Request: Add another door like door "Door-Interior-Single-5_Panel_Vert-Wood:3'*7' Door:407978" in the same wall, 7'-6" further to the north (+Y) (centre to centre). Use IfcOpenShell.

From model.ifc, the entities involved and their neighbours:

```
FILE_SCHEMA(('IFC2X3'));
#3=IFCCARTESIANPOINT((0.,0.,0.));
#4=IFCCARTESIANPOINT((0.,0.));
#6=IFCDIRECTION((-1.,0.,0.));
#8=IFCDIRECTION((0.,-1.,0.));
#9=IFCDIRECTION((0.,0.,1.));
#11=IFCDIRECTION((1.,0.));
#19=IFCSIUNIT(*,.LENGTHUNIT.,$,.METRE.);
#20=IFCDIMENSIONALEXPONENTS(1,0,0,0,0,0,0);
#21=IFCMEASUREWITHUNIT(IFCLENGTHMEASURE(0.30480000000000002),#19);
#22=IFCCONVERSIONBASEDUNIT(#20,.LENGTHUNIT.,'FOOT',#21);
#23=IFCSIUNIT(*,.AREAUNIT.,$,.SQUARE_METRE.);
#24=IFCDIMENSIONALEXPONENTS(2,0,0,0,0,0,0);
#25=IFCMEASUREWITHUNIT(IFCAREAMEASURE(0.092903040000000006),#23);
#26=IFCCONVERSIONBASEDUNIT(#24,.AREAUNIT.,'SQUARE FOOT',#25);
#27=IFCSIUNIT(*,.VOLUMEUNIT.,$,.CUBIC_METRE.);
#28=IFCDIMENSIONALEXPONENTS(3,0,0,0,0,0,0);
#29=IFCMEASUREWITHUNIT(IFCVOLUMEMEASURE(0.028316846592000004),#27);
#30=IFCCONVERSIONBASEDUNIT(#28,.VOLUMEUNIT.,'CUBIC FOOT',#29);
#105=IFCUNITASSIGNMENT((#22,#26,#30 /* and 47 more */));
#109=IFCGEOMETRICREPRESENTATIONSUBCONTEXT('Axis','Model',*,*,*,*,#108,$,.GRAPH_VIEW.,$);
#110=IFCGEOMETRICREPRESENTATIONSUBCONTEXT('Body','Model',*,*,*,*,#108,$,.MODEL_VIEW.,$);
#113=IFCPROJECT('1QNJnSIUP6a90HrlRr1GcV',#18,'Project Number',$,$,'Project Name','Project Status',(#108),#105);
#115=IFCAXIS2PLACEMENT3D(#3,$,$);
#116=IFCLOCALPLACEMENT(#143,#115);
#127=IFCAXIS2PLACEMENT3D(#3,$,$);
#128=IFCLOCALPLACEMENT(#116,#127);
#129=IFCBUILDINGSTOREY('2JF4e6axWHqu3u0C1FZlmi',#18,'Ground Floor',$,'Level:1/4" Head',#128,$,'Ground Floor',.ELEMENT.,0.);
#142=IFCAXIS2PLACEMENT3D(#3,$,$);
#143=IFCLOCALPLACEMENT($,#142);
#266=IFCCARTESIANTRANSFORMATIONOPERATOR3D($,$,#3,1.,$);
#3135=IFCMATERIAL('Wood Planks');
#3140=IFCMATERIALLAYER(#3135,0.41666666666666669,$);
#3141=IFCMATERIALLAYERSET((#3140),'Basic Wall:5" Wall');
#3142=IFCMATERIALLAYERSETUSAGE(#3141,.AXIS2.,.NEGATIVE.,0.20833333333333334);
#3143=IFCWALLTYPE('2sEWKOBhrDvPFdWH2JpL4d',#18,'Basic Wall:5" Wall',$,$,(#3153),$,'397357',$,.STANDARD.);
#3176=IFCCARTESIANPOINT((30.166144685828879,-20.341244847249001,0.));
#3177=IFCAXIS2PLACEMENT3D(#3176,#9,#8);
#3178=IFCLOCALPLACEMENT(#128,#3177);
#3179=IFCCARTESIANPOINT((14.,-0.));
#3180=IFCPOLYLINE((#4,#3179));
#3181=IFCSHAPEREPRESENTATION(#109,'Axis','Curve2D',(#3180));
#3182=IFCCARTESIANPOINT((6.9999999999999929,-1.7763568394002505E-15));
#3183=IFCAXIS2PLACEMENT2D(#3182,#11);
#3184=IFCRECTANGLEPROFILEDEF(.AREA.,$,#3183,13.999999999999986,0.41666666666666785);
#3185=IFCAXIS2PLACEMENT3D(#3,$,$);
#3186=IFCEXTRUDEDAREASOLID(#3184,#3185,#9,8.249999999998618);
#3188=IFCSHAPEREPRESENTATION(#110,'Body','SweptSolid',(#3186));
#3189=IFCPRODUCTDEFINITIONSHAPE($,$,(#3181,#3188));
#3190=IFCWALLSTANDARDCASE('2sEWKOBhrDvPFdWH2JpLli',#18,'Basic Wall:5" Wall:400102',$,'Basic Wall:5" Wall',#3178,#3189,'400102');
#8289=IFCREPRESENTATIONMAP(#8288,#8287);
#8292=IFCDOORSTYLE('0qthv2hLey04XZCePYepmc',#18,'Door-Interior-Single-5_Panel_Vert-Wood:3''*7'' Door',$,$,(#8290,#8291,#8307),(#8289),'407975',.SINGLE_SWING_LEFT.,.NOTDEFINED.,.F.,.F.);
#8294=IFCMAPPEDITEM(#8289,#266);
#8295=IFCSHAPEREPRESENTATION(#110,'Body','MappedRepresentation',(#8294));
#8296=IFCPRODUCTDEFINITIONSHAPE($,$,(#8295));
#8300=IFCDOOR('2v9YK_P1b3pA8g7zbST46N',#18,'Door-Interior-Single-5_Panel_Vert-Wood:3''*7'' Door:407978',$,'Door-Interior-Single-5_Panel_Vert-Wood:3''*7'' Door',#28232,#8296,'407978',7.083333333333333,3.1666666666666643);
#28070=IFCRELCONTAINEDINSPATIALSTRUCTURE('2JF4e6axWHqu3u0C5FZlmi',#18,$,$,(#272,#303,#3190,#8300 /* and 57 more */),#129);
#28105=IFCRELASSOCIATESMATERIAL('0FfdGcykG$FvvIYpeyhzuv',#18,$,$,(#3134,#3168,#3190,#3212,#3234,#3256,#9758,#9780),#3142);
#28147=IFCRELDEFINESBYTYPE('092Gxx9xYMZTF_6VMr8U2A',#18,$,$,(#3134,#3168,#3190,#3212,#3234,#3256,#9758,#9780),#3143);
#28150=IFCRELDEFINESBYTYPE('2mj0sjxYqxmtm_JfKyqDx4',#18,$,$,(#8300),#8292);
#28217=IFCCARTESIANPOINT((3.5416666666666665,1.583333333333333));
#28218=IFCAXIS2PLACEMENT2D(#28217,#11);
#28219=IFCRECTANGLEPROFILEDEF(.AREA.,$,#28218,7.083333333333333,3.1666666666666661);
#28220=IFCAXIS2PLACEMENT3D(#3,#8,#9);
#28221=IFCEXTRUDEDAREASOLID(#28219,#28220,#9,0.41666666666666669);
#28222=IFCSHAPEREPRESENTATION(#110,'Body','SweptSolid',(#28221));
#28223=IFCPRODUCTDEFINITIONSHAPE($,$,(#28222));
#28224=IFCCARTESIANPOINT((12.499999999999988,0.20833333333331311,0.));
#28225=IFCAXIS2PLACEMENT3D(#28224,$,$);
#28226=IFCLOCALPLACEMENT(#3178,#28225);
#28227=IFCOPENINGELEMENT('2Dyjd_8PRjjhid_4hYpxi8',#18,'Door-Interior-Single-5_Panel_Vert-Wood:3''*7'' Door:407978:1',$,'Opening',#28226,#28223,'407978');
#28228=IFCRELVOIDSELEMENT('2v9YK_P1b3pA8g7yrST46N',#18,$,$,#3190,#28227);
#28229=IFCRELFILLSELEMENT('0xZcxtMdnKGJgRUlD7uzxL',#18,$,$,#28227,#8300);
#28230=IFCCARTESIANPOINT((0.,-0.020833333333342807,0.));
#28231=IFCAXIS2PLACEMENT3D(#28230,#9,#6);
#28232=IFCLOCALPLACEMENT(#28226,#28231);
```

```python
import ifcopenshell
import ifcopenshell.api.feature
import ifcopenshell.api.geometry
import ifcopenshell.api.root
import ifcopenshell.geom
import ifcopenshell.util.element
import ifcopenshell.util.placement
import ifcopenshell.util.shape
import ifcopenshell.util.unit

model = ifcopenshell.open("model.ifc")
unit_scale = ifcopenshell.util.unit.calculate_unit_scale(model)
settings = ifcopenshell.geom.settings()


def volume(element):
    """Net volume in cubic metres, openings subtracted."""
    shape = ifcopenshell.geom.create_shape(settings, element)
    return ifcopenshell.util.shape.get_volume(shape.geometry)


def reuse_history(source, copy):
    """copy_class also copies each property set's owner history, people and application; keep the originals."""
    for rel in copy.IsDefinedBy:
        if rel.is_a("IfcRelDefinesByProperties") and (history := rel.RelatingPropertyDefinition.OwnerHistory):
            rel.RelatingPropertyDefinition.OwnerHistory = source.OwnerHistory
            ifcopenshell.util.element.remove_deep2(model, history)


door = model.by_guid("2v9YK_P1b3pA8g7zbST46N")
opening = door.FillsVoids[0].RelatingOpeningElement
wall = opening.VoidsElements[0].RelatingBuildingElement
before = volume(wall)
shift = ifcopenshell.util.placement.get_local_placement(wall.ObjectPlacement)[:3, 0] * -90 * 0.0254 / unit_scale

# copy_class copies the void relationship, type, container and properties, but no geometry.
new_opening = ifcopenshell.api.root.copy_class(model, product=opening)
new_opening.Representation = ifcopenshell.util.element.copy_deep(
    model, opening.Representation, exclude=["IfcGeometricRepresentationContext", "IfcRepresentationMap"]
)
new_opening.Name = "Door-Interior-Single-5_Panel_Vert-Wood:3'*7' Door"
new_opening.Tag = None
new_door = ifcopenshell.api.root.copy_class(model, product=door)
new_door.Representation = ifcopenshell.util.element.copy_deep(
    model, door.Representation, exclude=["IfcGeometricRepresentationContext", "IfcRepresentationMap"]
)
new_door.Name = "Door-Interior-Single-5_Panel_Vert-Wood:3'*7' Door"
new_door.Tag = None
reuse_history(door, new_door)
fills = ifcopenshell.api.feature.add_filling(model, opening=new_opening, element=new_door)
fills.OwnerHistory = new_door.OwnerHistory  # required in IFC2X3

for old, new in ((opening, new_opening), (door, new_door)):
    matrix = ifcopenshell.util.placement.get_local_placement(old.ObjectPlacement)
    matrix[:3, 3] += shift
    ifcopenshell.api.geometry.edit_object_placement(model, product=new, matrix=matrix, is_si=False)

after = volume(wall)

print(f"wall volume {before:.3f} -> {after:.3f} m3")

model.write("model_edited.ifc")
```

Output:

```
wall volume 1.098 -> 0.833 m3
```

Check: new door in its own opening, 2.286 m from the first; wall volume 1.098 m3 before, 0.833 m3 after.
